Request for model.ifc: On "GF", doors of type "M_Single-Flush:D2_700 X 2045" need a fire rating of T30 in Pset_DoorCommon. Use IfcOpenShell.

First a look at what the model holds.

```python
import ifcopenshell
import ifcopenshell.util.element

model = ifcopenshell.open("model.ifc")
print(model.schema)
storey = next(s for s in model.by_type("IfcBuildingStorey") if s.Name == "GF")
doors = [e for e in ifcopenshell.util.element.get_decomposition(storey) if e.is_a("IfcDoor")]
seen = {}
for e in doors:
    element_type = ifcopenshell.util.element.get_type(e)
    key = (element_type.Name if element_type != e and element_type else None, ifcopenshell.util.element.get_pset(e, "Pset_DoorCommon", "FireRating"))
    seen[key] = seen.get(key, 0) + 1
for (name, value), count in sorted(seen.items(), key=str):
    print(count, "x", name, "|", value)
```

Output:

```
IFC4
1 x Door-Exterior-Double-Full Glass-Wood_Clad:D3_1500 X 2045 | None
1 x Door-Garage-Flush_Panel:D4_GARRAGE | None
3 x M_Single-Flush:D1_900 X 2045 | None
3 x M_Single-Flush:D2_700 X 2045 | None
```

```python
import ifcopenshell
import ifcopenshell.api.pset
import ifcopenshell.util.element

model = ifcopenshell.open("model.ifc")

storey = next(s for s in model.by_type("IfcBuildingStorey") if s.Name == "GF")
doors = [e for e in ifcopenshell.util.element.get_decomposition(storey) if e.is_a("IfcDoor")]

count = 0
for e in doors:
    element_type = ifcopenshell.util.element.get_type(e)
    if element_type in (None, e) or element_type.Name != "M_Single-Flush:D2_700 X 2045":
        continue
    # add_pset returns the element's existing set when there is one.
    pset = ifcopenshell.api.pset.add_pset(model, product=e, name="Pset_DoorCommon")
    ifcopenshell.api.pset.edit_pset(model, pset=pset, properties={"FireRating": "T30"})
    count += 1

print(count, "doors updated")

model.write("model_edited.ifc")
```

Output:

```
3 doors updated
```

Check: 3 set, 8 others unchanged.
